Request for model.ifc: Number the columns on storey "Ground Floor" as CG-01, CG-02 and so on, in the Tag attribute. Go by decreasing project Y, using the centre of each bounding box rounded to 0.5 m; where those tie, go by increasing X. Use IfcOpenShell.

First a look at what the model holds.

```python
import ifcopenshell
import ifcopenshell.util.element
import ifcopenshell.util.placement

model = ifcopenshell.open("model.ifc")
print(model.schema)
storey = next(s for s in model.by_type("IfcBuildingStorey") if s.Name == "Ground Floor")
columns = [e for e in ifcopenshell.util.element.get_decomposition(storey) if e.is_a("IfcColumn")]
for e in sorted(columns, key=lambda e: e.id()):
    origin = ifcopenshell.util.placement.get_local_placement(e.ObjectPlacement)[:3, 3]
    print(e.id(), e.Tag, e.Name, origin.round(2) + 0.0, sep=" | ")
```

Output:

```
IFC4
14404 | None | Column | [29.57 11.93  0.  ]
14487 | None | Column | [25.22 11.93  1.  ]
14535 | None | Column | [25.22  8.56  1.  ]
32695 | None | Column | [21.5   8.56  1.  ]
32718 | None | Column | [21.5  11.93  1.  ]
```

```python
import ifcopenshell
import ifcopenshell.geom
import ifcopenshell.util.element
import ifcopenshell.util.shape

model = ifcopenshell.open("model.ifc")
settings = ifcopenshell.geom.settings()
settings.set("use-world-coords", True)


def centre(element):
    shape = ifcopenshell.geom.create_shape(settings, element)
    return ifcopenshell.util.shape.get_bbox_centroid(shape.geometry)


storey = next(s for s in model.by_type("IfcBuildingStorey") if s.Name == "Ground Floor")
columns = [e for e in ifcopenshell.util.element.get_decomposition(storey) if e.is_a("IfcColumn")]

# Insertion points can sit at a corner or the storey origin, so sort by the geometry (in metres).
centres = {e: centre(e) for e in columns}
columns.sort(key=lambda e: (-round(centres[e][1] / 0.5), centres[e][0]))

for i, e in enumerate(columns, start=1):
    number = f"CG-{i:02d}"
    e.Tag = number
    print(e.id(), number)

model.write("model_rev.ifc")
```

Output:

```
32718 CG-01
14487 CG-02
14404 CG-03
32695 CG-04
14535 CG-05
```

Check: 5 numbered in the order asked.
